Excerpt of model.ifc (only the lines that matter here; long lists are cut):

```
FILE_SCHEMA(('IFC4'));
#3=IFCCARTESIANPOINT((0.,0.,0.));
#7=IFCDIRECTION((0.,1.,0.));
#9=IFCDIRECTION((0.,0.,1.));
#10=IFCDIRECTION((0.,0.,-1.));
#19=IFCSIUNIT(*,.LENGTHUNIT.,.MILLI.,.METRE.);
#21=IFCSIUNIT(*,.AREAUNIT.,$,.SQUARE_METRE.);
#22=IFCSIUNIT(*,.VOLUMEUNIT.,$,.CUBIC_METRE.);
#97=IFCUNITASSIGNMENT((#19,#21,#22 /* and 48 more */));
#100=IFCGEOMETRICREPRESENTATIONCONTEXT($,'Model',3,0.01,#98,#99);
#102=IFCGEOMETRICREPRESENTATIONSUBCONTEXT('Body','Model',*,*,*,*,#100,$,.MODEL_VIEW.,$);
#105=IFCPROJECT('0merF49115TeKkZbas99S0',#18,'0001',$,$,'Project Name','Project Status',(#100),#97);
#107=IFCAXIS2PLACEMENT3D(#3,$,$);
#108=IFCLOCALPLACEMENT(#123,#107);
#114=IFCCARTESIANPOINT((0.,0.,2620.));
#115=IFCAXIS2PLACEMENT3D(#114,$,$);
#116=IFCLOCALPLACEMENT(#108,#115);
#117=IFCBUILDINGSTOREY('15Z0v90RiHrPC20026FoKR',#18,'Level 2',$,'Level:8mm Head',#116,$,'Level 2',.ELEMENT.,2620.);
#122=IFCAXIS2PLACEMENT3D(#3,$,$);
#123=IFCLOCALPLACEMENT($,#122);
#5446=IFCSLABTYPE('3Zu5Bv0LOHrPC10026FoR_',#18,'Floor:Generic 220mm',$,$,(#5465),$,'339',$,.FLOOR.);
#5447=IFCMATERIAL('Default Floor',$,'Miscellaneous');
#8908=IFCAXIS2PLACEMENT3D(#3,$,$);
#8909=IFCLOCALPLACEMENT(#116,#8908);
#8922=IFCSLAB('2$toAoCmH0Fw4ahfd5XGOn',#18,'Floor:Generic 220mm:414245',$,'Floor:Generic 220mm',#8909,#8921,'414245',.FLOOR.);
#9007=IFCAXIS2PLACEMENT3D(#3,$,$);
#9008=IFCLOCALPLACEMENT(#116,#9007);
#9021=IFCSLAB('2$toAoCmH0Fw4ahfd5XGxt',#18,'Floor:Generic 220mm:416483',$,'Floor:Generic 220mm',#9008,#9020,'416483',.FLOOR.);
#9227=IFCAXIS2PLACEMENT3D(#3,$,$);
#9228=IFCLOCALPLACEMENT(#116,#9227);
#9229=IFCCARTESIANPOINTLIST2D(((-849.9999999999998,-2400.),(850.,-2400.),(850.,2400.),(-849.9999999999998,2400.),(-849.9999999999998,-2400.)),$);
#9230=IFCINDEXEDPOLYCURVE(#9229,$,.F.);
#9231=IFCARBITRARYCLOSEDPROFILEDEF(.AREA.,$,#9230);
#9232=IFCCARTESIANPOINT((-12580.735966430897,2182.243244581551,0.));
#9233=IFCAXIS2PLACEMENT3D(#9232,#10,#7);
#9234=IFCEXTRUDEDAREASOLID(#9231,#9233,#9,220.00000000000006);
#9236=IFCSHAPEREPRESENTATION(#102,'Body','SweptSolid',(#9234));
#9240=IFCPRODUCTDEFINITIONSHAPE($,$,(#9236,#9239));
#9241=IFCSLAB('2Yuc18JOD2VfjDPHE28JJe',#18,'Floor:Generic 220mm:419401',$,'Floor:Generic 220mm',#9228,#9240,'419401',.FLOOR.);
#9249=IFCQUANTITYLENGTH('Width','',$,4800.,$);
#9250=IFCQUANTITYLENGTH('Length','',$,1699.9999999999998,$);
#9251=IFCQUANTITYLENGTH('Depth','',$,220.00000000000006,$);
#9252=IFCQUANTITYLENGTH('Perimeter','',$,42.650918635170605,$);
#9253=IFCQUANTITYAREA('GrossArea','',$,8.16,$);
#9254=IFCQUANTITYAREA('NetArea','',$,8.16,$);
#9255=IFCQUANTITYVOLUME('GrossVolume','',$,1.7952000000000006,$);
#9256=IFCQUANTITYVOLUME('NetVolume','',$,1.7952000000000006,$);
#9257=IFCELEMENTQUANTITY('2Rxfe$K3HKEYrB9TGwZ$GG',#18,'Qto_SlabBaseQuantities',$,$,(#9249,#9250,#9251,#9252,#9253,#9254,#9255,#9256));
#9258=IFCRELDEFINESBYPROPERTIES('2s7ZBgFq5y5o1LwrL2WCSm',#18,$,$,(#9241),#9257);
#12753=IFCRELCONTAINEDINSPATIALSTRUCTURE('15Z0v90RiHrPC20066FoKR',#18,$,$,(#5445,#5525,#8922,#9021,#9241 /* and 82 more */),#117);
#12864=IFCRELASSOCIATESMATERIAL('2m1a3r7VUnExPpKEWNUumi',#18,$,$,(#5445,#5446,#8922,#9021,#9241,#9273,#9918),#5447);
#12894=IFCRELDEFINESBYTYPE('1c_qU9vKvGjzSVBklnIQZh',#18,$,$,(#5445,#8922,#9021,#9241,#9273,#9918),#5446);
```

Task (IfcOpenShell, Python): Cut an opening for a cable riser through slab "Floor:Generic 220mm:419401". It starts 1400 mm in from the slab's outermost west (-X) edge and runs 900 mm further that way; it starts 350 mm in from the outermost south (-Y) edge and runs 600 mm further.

```python
import numpy as np
import ifcopenshell
import ifcopenshell.api.feature
import ifcopenshell.api.geometry
import ifcopenshell.api.pset
import ifcopenshell.api.root
import ifcopenshell.geom
import ifcopenshell.util.element
import ifcopenshell.util.placement
import ifcopenshell.util.representation
import ifcopenshell.util.shape
import ifcopenshell.util.unit

model = ifcopenshell.open("model.ifc")
unit_scale = ifcopenshell.util.unit.calculate_unit_scale(model)
area_scale = ifcopenshell.util.unit.calculate_unit_scale(model, "AREAUNIT")
volume_scale = ifcopenshell.util.unit.calculate_unit_scale(model, "VOLUMEUNIT")
settings = ifcopenshell.geom.settings()


def volume(element):
    """Net volume in cubic metres, openings subtracted."""
    shape = ifcopenshell.geom.create_shape(settings, element)
    return ifcopenshell.util.shape.get_volume(shape.geometry)


slab = model.by_guid("2Yuc18JOD2VfjDPHE28JJe")
before = volume(slab)

# Extent in the slab's own axes, in metres. The edges named are its -X and -Y sides.
slab_shape = ifcopenshell.geom.create_shape(settings, slab)
vertices = ifcopenshell.util.shape.get_vertices(slab_shape.geometry)
x_min, y_min, bottom = vertices.min(axis=0)
top = vertices[:, 2].max()

opening = ifcopenshell.api.root.create_entity(model, ifc_class="IfcOpeningElement", name="Cable riser opening", predefined_type="OPENING")
context = ifcopenshell.util.representation.get_context(model, "Model", "Body", "MODEL_VIEW")
width, depth = 0.9, 0.6
outline = [(0.0, 0.0), (width, 0.0), (width, depth), (0.0, depth), (0.0, 0.0)]
# Overshoot both faces by 50 mm so the cut is clean.
shape = ifcopenshell.api.geometry.add_slab_representation(
    model, context=context, depth=top - bottom + 0.1, polyline=outline
)
ifcopenshell.api.geometry.assign_representation(model, product=opening, representation=shape)

matrix = ifcopenshell.util.placement.get_local_placement(slab.ObjectPlacement)
matrix[:, 3] = matrix @ np.append(np.array([x_min + 1.4, y_min + 0.35, bottom - 0.05]) / unit_scale, 1.0)
ifcopenshell.api.geometry.edit_object_placement(model, product=opening, matrix=matrix, is_si=False)
ifcopenshell.api.feature.add_feature(model, feature=opening, element=slab)

after = volume(slab)

# Update the slab's stored quantities.
qto = model.by_id(ifcopenshell.util.element.get_pset(slab, "Qto_SlabBaseQuantities", should_inherit=False)["id"])
ifcopenshell.api.pset.edit_qto(model, qto=qto, properties={
    "NetArea": after / (top - bottom) / area_scale,
    "NetVolume": after / volume_scale,
})

print(f"slab volume {before:.3f} -> {after:.3f} m3")

model.write("model-out.ifc")
```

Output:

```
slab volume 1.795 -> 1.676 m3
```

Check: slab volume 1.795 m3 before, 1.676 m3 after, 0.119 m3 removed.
